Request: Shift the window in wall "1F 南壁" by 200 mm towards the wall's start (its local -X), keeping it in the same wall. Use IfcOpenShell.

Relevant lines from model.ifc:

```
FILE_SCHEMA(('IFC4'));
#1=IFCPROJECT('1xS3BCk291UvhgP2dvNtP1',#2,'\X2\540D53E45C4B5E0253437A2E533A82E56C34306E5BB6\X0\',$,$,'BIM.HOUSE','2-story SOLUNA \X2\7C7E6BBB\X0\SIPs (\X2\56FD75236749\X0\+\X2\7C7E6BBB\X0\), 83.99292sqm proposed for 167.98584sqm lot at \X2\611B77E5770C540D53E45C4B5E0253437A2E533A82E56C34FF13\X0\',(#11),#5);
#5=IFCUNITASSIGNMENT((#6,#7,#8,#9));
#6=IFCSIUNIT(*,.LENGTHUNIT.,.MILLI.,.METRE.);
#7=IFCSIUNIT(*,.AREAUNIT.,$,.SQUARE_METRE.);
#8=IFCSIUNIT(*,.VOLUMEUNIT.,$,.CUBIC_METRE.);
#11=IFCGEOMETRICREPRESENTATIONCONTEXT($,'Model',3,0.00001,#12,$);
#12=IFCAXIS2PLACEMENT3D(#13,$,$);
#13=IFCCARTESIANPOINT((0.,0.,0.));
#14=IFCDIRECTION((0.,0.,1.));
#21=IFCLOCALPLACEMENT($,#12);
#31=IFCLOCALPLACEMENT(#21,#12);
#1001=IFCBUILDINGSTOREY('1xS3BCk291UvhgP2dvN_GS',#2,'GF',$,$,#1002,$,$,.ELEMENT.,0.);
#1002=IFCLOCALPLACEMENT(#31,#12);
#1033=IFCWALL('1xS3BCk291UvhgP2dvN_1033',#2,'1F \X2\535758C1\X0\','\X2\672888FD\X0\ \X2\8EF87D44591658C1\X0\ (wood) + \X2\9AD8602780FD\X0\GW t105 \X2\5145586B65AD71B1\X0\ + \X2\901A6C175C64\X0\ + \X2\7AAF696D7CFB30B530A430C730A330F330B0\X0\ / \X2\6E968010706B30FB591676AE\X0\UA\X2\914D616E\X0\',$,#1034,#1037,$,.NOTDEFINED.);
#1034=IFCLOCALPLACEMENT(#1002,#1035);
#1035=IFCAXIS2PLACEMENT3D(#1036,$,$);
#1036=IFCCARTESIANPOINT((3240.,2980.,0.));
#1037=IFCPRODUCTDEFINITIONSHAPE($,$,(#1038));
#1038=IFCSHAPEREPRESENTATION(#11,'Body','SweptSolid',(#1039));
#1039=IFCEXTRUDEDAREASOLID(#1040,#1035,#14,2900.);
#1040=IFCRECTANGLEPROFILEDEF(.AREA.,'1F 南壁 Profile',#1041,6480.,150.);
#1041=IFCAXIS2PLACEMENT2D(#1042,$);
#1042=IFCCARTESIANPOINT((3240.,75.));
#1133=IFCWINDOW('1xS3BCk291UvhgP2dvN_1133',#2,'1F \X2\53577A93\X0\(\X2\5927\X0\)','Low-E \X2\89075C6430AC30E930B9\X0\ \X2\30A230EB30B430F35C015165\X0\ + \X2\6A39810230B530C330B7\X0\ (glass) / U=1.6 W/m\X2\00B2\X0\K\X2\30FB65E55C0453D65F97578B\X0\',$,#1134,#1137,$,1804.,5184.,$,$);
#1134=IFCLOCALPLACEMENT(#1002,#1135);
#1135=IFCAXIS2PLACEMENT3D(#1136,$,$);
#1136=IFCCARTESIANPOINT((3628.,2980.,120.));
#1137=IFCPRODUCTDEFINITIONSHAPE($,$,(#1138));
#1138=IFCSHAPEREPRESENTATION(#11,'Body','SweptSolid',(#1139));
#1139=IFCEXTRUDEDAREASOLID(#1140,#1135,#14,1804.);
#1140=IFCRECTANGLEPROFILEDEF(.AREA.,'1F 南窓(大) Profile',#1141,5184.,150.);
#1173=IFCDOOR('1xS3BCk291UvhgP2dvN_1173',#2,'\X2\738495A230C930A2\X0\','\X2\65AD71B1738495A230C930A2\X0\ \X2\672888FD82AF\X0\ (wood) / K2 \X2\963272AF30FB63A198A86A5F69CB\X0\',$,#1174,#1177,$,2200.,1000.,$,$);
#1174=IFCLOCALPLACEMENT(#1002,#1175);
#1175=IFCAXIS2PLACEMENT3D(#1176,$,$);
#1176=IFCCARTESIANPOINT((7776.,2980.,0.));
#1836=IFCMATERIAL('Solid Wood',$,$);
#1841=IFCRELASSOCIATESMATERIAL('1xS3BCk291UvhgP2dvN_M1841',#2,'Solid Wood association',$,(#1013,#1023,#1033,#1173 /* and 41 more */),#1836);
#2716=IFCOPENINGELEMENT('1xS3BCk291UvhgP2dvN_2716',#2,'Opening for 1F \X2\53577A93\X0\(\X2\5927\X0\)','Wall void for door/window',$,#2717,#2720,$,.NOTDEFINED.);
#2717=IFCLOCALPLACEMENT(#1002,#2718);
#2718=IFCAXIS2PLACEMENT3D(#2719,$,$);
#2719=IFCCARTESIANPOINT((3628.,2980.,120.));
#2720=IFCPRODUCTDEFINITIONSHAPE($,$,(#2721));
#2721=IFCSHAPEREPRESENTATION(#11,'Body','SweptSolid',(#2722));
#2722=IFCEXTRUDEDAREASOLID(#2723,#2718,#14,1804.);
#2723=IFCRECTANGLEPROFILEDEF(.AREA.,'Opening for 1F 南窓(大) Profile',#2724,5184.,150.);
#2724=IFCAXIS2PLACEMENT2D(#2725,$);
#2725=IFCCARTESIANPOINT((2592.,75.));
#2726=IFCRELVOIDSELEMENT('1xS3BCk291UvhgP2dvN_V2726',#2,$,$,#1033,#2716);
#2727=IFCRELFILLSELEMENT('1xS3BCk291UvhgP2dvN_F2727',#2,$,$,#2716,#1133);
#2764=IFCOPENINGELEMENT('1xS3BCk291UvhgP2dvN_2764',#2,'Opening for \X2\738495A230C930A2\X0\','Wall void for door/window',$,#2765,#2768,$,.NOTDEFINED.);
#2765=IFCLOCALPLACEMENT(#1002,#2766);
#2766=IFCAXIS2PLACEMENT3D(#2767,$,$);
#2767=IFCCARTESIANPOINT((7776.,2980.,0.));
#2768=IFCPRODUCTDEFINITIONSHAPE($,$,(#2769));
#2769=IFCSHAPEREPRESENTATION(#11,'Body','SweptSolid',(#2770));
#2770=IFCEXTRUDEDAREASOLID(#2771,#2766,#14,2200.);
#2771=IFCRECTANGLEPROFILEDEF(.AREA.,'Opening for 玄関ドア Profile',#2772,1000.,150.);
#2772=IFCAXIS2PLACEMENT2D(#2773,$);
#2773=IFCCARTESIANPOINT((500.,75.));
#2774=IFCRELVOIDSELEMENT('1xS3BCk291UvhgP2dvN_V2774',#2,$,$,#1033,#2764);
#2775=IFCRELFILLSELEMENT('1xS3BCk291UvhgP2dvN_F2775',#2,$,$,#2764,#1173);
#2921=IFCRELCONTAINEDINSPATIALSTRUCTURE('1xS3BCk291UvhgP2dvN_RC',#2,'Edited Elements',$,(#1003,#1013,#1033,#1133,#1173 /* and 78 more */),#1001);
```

```python
import ifcopenshell
import ifcopenshell.api.geometry
import ifcopenshell.util.placement
import ifcopenshell.util.unit

model = ifcopenshell.open("model.ifc")
unit_scale = ifcopenshell.util.unit.calculate_unit_scale(model)

window = model.by_guid("1xS3BCk291UvhgP2dvN_1133")
opening = window.FillsVoids[0].RelatingOpeningElement
wall = opening.VoidsElements[0].RelatingBuildingElement

wall_matrix = ifcopenshell.util.placement.get_local_placement(wall.ObjectPlacement)
shift = wall_matrix[:3, 0] * -0.2 / unit_scale
before = ifcopenshell.util.placement.get_local_placement(window.ObjectPlacement)[:3, 3].copy()

# The window is not placed relative to its opening, so move both.
for product in (opening, window):
    matrix = ifcopenshell.util.placement.get_local_placement(product.ObjectPlacement)
    matrix[:3, 3] += shift
    ifcopenshell.api.geometry.edit_object_placement(model, product=product, matrix=matrix, is_si=False)

after = ifcopenshell.util.placement.get_local_placement(window.ObjectPlacement)[:3, 3]
print("window moved by", (after - before).round(3) + 0.0)

model.write("model_v2.ifc")
```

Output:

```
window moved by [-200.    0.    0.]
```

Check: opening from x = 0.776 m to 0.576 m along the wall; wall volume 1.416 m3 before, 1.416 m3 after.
